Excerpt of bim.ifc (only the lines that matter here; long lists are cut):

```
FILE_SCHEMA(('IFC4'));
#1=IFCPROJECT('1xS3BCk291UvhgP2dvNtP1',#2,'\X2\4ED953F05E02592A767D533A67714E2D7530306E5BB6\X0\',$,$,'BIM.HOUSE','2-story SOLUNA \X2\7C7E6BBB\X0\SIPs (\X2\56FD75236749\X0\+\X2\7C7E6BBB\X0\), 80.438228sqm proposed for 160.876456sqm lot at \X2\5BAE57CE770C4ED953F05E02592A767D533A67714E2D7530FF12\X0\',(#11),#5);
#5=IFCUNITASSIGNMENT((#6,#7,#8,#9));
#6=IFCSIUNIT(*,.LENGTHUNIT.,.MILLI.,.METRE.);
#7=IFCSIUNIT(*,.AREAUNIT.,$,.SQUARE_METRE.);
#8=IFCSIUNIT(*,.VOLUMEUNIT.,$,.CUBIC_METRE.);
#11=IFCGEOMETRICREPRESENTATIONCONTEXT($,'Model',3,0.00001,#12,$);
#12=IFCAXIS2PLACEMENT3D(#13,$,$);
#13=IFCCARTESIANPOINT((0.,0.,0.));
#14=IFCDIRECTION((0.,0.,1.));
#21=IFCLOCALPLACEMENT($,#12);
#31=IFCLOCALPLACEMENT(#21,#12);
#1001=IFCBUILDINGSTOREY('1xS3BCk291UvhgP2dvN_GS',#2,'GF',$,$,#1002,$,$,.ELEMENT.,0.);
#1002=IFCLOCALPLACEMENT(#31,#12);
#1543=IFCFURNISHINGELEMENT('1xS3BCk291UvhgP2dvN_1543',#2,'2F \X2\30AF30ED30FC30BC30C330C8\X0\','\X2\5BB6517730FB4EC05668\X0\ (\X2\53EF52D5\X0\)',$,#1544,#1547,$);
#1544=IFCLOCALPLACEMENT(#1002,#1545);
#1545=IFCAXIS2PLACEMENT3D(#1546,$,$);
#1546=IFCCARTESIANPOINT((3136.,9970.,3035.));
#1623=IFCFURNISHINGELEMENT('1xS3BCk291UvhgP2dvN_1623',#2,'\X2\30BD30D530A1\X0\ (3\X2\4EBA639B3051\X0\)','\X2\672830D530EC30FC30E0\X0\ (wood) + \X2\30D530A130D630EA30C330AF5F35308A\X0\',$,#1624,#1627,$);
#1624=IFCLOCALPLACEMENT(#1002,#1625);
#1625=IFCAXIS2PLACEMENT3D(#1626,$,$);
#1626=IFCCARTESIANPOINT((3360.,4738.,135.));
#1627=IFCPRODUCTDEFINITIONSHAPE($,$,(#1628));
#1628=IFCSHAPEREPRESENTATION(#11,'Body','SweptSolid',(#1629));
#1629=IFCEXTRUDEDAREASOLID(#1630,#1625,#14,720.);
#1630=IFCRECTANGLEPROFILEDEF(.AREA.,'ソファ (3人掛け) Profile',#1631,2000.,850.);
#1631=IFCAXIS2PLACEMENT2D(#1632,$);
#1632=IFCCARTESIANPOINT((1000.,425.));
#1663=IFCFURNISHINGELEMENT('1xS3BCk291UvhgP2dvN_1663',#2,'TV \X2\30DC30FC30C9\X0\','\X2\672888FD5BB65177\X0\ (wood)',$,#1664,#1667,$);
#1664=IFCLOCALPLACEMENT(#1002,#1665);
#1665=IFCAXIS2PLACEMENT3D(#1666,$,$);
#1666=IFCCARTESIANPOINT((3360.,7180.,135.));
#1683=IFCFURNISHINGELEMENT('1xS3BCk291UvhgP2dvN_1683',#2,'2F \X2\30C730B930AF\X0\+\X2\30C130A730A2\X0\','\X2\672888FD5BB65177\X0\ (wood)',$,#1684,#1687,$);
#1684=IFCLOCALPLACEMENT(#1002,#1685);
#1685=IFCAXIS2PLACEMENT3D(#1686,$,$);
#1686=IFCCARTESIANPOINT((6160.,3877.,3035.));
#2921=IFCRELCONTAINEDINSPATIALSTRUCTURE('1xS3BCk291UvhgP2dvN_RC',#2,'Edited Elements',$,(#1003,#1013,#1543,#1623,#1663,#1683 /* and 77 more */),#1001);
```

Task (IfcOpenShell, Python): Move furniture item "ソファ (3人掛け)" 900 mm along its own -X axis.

```python
import ifcopenshell
import ifcopenshell.api.geometry
import ifcopenshell.util.placement
import ifcopenshell.util.unit

model = ifcopenshell.open("bim.ifc")
unit_scale = ifcopenshell.util.unit.calculate_unit_scale(model)

item = model.by_guid("1xS3BCk291UvhgP2dvN_1623")
matrix = ifcopenshell.util.placement.get_local_placement(item.ObjectPlacement)
matrix[:3, 3] -= matrix[:3, 0] * 0.9 / unit_scale
ifcopenshell.api.geometry.edit_object_placement(model, product=item, matrix=matrix, is_si=False)

print(ifcopenshell.util.placement.get_local_placement(item.ObjectPlacement).round(3) + 0.0)

model.write("bim-out.ifc")
```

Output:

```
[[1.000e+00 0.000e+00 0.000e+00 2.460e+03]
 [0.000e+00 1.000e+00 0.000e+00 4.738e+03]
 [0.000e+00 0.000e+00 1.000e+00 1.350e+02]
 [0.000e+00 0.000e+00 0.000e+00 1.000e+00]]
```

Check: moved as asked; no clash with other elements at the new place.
